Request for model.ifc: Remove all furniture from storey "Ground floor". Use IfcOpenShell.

First a look at what the model holds.

```python
import ifcopenshell
import ifcopenshell.util.element

model = ifcopenshell.open("model.ifc")
print(model.schema)
storey = next(s for s in model.by_type("IfcBuildingStorey") if s.Name == "Ground floor")
furniture = [e for e in ifcopenshell.util.element.get_decomposition(storey) if e.is_a("IfcFurnishingElement")]
seen = {}
for e in furniture:
    element_type = ifcopenshell.util.element.get_type(e)
    name = element_type.Name if element_type not in (None, e) else None
    seen[name] = seen.get(name, 0) + 1
for name, count in sorted(seen.items(), key=str):
    print(count, "x", name)
```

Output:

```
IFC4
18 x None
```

```python
import ifcopenshell
import ifcopenshell.api.root
import ifcopenshell.util.element

model = ifcopenshell.open("model.ifc")

storey = next(s for s in model.by_type("IfcBuildingStorey") if s.Name == "Ground floor")
furniture = [e for e in ifcopenshell.util.element.get_decomposition(storey) if e.is_a("IfcFurnishingElement")]

for e in furniture:
    ifcopenshell.api.root.remove_product(model, product=e)
print(len(furniture), "removed")

model.write("model-out.ifc")
```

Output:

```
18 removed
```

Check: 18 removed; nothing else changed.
